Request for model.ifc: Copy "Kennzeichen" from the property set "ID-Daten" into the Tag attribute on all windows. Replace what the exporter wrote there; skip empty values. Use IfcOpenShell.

First a look at what the model holds.

```python
import ifcopenshell
import ifcopenshell.util.element

model = ifcopenshell.open("model.ifc")
print(model.schema)
windows = model.by_type("IfcWindow")
print(len(windows), "windows")
for e in windows[:8]:
    source = ifcopenshell.util.element.get_pset(e, "ID-Daten", "Kennzeichen")
    target = e.Tag
    print(e.id(), repr(source), repr(target), sep=" | ")
```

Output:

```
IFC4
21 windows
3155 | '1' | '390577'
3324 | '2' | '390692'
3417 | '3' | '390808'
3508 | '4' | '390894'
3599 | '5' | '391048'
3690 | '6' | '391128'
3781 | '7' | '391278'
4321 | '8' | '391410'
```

```python
import ifcopenshell
import ifcopenshell.util.element

model = ifcopenshell.open("model.ifc")

count = 0
for e in model.by_type("IfcWindow"):
    value = ifcopenshell.util.element.get_pset(e, "ID-Daten", "Kennzeichen")
    current = e.Tag
    if not value or not value.strip() or current == value:
        continue
    e.Tag = value
    count += 1

print(count, "windows updated")

model.write("model_rev.ifc")
```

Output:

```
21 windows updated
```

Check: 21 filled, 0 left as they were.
